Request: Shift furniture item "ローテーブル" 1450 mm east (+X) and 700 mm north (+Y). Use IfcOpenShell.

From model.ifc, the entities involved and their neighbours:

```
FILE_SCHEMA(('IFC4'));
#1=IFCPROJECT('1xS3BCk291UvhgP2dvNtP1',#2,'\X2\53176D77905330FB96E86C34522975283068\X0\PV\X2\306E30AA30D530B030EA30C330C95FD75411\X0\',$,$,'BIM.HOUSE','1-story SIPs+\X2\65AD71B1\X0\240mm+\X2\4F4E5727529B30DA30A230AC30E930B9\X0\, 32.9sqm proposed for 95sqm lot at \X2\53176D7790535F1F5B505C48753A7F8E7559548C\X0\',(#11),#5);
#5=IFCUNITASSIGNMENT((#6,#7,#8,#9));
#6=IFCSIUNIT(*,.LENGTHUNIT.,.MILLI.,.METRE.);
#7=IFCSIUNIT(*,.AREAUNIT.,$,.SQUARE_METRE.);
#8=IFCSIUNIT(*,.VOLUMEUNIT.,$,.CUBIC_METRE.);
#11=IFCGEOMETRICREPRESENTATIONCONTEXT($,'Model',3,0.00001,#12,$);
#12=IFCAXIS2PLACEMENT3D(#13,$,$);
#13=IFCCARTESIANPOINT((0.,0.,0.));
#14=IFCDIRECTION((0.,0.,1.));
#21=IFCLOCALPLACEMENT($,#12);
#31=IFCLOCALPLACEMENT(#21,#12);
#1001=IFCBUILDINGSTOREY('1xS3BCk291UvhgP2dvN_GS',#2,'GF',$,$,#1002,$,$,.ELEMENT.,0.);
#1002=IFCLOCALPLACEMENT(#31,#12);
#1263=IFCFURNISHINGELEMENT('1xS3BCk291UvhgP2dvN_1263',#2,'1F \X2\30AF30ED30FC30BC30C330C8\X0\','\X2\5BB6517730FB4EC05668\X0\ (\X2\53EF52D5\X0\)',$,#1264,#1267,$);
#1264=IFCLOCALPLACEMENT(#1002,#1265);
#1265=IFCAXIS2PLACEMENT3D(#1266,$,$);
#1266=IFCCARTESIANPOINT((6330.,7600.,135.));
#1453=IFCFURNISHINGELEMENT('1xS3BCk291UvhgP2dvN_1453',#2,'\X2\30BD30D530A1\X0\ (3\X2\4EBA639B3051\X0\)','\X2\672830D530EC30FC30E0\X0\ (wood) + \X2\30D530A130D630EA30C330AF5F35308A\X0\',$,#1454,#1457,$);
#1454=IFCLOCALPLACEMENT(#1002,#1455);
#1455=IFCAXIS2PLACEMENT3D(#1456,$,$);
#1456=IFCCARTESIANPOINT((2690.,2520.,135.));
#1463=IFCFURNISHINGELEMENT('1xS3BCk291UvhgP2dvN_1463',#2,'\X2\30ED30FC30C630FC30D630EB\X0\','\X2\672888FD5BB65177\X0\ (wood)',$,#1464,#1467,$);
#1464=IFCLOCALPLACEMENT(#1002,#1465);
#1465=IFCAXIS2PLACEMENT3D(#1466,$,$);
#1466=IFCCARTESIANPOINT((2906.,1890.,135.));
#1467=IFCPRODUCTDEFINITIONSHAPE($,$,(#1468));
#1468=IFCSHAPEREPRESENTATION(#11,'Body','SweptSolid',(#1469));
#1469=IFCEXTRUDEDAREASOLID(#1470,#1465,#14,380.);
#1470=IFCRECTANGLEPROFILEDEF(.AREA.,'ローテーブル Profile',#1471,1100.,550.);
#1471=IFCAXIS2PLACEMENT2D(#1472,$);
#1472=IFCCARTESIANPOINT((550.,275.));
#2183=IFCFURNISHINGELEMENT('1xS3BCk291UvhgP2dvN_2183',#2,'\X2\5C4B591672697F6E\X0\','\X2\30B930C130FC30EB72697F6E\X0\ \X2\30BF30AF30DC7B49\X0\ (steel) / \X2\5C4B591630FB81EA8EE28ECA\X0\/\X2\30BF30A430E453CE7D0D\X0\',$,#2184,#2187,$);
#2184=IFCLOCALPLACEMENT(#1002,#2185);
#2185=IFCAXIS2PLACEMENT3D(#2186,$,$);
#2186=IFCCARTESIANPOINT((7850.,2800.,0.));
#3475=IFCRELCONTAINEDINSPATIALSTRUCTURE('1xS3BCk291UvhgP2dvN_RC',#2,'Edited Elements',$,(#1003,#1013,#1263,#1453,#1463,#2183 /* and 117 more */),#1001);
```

```python
import ifcopenshell
import ifcopenshell.api.geometry
import ifcopenshell.util.placement
import ifcopenshell.util.unit

model = ifcopenshell.open("model.ifc")
unit_scale = ifcopenshell.util.unit.calculate_unit_scale(model)

item = model.by_id(1463)
matrix = ifcopenshell.util.placement.get_local_placement(item.ObjectPlacement)
matrix[0, 3] += 1.45 / unit_scale
matrix[1, 3] += 0.7 / unit_scale
ifcopenshell.api.geometry.edit_object_placement(model, product=item, matrix=matrix, is_si=False)

print(ifcopenshell.util.placement.get_local_placement(item.ObjectPlacement).round(3) + 0.0)

model.write("model_updated.ifc")
```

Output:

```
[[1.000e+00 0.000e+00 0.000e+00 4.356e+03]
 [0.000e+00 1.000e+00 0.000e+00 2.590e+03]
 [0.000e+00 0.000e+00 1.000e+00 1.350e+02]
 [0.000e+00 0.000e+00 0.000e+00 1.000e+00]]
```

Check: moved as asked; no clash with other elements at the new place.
